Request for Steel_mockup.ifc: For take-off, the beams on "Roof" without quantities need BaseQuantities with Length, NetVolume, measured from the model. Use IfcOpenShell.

First a look at what the model holds.

```python
import ifcopenshell
import ifcopenshell.util.element
import ifcopenshell.util.unit

model = ifcopenshell.open("Steel_mockup.ifc")
print(model.schema)
for unit_type in ("LENGTHUNIT", "AREAUNIT", "VOLUMEUNIT"):
    print(unit_type, ifcopenshell.util.unit.calculate_unit_scale(model, unit_type))
storey = next(s for s in model.by_type("IfcBuildingStorey") if s.Name == "Roof")
beams = [e for e in ifcopenshell.util.element.get_decomposition(storey) if e.is_a("IfcBeam")]
for e in sorted(beams, key=lambda e: e.id()):
    print(e.id(), e.is_a(), e.Name, list(ifcopenshell.util.element.get_psets(e, qtos_only=True)), sep=" | ")
```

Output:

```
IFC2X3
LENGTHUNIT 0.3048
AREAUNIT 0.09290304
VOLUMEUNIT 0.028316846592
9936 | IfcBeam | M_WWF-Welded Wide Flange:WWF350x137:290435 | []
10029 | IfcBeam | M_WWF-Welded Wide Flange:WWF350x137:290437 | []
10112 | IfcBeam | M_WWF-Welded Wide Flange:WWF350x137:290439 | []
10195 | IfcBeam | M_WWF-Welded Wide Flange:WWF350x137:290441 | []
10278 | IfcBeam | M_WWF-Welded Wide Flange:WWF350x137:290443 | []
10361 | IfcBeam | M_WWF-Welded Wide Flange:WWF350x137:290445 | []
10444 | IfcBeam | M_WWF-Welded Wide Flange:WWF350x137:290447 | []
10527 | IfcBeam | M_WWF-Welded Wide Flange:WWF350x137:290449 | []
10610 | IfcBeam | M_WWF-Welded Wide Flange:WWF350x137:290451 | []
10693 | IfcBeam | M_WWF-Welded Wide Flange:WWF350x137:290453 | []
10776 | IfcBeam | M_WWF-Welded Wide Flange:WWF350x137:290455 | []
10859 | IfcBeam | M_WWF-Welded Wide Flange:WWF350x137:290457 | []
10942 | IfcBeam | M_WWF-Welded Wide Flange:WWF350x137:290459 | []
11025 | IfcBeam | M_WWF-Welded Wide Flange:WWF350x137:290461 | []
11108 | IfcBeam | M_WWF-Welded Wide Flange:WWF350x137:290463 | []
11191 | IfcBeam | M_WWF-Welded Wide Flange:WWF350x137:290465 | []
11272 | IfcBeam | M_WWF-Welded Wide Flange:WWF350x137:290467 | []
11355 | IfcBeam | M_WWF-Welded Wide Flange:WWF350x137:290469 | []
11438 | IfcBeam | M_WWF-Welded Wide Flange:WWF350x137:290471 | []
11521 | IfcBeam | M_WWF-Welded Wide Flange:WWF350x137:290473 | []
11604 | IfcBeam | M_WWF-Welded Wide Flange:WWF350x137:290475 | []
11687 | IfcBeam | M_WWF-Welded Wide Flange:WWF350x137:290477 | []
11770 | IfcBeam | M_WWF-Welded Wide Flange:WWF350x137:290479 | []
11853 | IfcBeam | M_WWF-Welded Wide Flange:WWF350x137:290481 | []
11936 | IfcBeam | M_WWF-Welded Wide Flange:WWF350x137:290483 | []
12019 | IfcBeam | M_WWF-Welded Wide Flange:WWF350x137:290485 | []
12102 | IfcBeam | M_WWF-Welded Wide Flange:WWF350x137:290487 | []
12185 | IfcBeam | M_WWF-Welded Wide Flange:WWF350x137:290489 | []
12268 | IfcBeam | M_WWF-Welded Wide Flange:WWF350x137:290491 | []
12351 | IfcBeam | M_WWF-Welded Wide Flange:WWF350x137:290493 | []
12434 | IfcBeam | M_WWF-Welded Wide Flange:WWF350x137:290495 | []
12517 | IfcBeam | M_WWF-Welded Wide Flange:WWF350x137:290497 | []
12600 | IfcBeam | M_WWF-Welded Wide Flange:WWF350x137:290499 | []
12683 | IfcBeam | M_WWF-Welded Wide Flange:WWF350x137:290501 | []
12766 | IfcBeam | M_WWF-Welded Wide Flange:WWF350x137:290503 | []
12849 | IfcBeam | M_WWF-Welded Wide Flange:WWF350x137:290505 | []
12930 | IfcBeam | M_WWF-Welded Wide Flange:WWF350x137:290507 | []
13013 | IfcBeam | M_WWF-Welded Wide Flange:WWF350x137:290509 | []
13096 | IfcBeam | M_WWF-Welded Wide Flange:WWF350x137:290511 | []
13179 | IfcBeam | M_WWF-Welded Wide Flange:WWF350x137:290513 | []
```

```python
import ifcopenshell
import ifcopenshell.api.pset
import ifcopenshell.geom
import ifcopenshell.util.element
import ifcopenshell.util.shape
import ifcopenshell.util.unit

model = ifcopenshell.open("Steel_mockup.ifc")
unit_scale = ifcopenshell.util.unit.calculate_unit_scale(model)
volume_scale = ifcopenshell.util.unit.calculate_unit_scale(model, "VOLUMEUNIT")
settings = ifcopenshell.geom.settings()

storey = next(s for s in model.by_type("IfcBuildingStorey") if s.Name == "Roof")
beams = [e for e in ifcopenshell.util.element.get_decomposition(storey) if e.is_a("IfcBeam")]

for e in sorted(beams, key=lambda e: e.id()):
    if ifcopenshell.util.element.get_psets(e, qtos_only=True, should_inherit=False):
        continue
    # Geometry comes back in metres, in the element's own axes.
    shape = ifcopenshell.geom.create_shape(settings, e)
    values = {
        "Length": ifcopenshell.util.shape.get_max_xyz(shape.geometry) / unit_scale,
        "NetVolume": ifcopenshell.util.shape.get_volume(shape.geometry) / volume_scale,
    }
    qto = ifcopenshell.api.pset.add_qto(model, product=e, name="BaseQuantities")
    ifcopenshell.api.pset.edit_qto(model, qto=qto, properties=values)
    print(e.id(), {k: round(v, 3) for k, v in values.items()})

model.write("Steel_mockup_v2.ifc")
```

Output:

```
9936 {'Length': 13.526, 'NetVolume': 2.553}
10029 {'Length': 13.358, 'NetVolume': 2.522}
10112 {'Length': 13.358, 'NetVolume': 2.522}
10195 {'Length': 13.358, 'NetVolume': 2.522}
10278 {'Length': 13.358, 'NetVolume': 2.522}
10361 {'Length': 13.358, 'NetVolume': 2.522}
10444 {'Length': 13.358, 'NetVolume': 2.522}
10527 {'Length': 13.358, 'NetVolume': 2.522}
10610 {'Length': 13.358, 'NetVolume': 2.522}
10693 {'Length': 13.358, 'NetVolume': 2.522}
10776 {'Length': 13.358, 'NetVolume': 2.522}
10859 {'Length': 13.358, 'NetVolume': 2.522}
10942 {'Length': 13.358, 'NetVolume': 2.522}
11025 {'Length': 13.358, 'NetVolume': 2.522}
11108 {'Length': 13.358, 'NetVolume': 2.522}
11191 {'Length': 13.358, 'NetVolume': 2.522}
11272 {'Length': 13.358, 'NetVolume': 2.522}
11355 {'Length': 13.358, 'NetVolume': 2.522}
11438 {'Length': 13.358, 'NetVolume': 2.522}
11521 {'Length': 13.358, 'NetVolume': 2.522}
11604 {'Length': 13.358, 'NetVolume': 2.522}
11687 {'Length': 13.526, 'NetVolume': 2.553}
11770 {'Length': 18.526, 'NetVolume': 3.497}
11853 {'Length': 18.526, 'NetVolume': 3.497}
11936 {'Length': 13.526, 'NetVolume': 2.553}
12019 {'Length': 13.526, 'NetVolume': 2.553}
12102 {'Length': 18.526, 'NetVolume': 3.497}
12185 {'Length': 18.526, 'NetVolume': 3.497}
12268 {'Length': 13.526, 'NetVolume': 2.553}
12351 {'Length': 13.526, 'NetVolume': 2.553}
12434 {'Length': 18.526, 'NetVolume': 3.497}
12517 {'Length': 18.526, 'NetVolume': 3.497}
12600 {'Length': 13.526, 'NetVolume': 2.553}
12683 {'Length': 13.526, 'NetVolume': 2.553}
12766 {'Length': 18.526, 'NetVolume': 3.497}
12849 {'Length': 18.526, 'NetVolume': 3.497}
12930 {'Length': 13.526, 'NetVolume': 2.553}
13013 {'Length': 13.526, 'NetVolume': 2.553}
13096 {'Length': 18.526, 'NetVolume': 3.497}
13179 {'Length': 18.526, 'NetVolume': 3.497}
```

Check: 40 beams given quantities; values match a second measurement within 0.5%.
